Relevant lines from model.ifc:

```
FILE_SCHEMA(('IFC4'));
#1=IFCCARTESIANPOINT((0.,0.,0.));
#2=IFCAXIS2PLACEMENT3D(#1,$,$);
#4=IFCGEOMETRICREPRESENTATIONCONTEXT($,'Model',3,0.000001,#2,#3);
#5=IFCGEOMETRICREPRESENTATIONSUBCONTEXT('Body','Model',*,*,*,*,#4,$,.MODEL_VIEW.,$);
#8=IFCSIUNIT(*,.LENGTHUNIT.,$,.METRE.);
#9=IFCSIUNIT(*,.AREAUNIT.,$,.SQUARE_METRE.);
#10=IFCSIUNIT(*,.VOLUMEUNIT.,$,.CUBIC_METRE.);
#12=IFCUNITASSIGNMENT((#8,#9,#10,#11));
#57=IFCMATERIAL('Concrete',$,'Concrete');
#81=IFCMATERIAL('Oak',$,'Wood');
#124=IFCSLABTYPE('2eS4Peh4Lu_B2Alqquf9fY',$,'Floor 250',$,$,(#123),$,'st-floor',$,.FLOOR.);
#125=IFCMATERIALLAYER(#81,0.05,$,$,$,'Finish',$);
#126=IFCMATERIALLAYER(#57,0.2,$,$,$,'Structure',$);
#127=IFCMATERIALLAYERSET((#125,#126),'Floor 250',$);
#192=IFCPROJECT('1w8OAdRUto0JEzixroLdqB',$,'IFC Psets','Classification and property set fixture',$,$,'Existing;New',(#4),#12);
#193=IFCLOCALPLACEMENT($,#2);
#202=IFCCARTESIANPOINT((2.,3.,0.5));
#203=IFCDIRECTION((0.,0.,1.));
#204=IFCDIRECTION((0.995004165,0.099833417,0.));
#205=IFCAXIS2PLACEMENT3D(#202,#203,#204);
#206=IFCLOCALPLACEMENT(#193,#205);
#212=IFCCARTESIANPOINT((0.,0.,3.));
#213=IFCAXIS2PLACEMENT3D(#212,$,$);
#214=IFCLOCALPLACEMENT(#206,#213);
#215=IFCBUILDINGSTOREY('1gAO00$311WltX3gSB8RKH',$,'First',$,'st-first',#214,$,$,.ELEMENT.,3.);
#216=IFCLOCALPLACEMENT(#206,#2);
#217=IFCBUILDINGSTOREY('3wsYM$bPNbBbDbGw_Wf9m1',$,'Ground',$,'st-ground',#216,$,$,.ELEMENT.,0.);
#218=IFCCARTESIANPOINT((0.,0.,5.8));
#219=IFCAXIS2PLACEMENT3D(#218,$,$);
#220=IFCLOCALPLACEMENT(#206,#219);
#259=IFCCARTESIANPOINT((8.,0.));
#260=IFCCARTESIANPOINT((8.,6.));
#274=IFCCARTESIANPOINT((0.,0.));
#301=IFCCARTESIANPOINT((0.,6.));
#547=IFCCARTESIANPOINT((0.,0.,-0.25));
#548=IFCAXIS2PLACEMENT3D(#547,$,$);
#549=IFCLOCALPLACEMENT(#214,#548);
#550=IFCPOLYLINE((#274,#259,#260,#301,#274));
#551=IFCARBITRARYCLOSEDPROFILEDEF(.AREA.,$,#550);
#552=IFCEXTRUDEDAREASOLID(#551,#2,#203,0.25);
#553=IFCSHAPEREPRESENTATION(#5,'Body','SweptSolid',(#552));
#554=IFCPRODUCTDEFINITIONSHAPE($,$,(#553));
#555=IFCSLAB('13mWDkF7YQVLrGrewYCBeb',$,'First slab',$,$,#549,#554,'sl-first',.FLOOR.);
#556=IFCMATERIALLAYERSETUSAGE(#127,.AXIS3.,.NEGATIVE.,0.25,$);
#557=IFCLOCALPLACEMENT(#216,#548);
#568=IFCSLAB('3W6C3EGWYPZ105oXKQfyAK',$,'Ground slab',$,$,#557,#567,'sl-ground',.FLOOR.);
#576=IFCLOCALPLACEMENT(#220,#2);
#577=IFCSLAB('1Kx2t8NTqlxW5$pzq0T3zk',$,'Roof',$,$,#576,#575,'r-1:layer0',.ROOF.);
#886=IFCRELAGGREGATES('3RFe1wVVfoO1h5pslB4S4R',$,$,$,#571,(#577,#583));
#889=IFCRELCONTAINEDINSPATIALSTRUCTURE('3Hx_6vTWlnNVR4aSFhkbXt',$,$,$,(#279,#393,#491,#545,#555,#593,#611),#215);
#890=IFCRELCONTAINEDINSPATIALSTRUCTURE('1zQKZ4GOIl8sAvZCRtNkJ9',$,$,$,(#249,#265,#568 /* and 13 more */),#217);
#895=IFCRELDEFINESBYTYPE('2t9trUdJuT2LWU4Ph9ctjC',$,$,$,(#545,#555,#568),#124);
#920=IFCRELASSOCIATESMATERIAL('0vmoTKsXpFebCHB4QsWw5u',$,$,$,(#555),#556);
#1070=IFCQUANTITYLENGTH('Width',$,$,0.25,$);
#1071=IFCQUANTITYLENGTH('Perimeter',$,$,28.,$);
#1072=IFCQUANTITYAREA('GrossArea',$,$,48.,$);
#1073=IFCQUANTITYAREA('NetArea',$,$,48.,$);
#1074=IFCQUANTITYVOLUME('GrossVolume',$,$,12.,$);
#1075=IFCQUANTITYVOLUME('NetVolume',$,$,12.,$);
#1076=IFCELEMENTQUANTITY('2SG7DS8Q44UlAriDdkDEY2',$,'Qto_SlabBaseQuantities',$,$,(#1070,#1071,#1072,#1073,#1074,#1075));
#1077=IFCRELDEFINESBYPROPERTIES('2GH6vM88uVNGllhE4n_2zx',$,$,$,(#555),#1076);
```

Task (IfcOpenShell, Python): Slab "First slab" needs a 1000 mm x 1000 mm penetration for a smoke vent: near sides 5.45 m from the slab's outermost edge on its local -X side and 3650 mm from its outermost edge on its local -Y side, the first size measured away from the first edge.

```python
import numpy as np
import ifcopenshell
import ifcopenshell.api.feature
import ifcopenshell.api.geometry
import ifcopenshell.api.pset
import ifcopenshell.api.root
import ifcopenshell.geom
import ifcopenshell.util.element
import ifcopenshell.util.placement
import ifcopenshell.util.representation
import ifcopenshell.util.shape
import ifcopenshell.util.unit

model = ifcopenshell.open("model.ifc")
unit_scale = ifcopenshell.util.unit.calculate_unit_scale(model)
area_scale = ifcopenshell.util.unit.calculate_unit_scale(model, "AREAUNIT")
volume_scale = ifcopenshell.util.unit.calculate_unit_scale(model, "VOLUMEUNIT")
settings = ifcopenshell.geom.settings()


def volume(element):
    """Net volume in cubic metres, openings subtracted."""
    shape = ifcopenshell.geom.create_shape(settings, element)
    return ifcopenshell.util.shape.get_volume(shape.geometry)


slab = model.by_guid("13mWDkF7YQVLrGrewYCBeb")
before = volume(slab)

# Extent in the slab's own axes, in metres. The edges named are its -X and -Y sides.
slab_shape = ifcopenshell.geom.create_shape(settings, slab)
vertices = ifcopenshell.util.shape.get_vertices(slab_shape.geometry)
x_min, y_min, bottom = vertices.min(axis=0)
top = vertices[:, 2].max()

opening = ifcopenshell.api.root.create_entity(model, ifc_class="IfcOpeningElement", name="Smoke vent opening", predefined_type="OPENING")
context = ifcopenshell.util.representation.get_context(model, "Model", "Body", "MODEL_VIEW")
width, depth = 1, 1
outline = [(0.0, 0.0), (width, 0.0), (width, depth), (0.0, depth), (0.0, 0.0)]
# Overshoot both faces by 50 mm so the cut is clean.
shape = ifcopenshell.api.geometry.add_slab_representation(
    model, context=context, depth=top - bottom + 0.1, polyline=outline
)
ifcopenshell.api.geometry.assign_representation(model, product=opening, representation=shape)

matrix = ifcopenshell.util.placement.get_local_placement(slab.ObjectPlacement)
matrix[:, 3] = matrix @ np.append(np.array([x_min + 5.45, y_min + 3.65, bottom - 0.05]) / unit_scale, 1.0)
ifcopenshell.api.geometry.edit_object_placement(model, product=opening, matrix=matrix, is_si=False)
ifcopenshell.api.feature.add_feature(model, feature=opening, element=slab)

after = volume(slab)

# Update the slab's stored quantities.
qto = model.by_id(ifcopenshell.util.element.get_pset(slab, "Qto_SlabBaseQuantities", should_inherit=False)["id"])
ifcopenshell.api.pset.edit_qto(model, qto=qto, properties={
    "NetArea": after / (top - bottom) / area_scale,
    "NetVolume": after / volume_scale,
})

print(f"slab volume {before:.3f} -> {after:.3f} m3")

model.write("model_rev.ifc")
```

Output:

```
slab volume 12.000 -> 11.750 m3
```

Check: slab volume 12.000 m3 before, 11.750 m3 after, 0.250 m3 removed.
